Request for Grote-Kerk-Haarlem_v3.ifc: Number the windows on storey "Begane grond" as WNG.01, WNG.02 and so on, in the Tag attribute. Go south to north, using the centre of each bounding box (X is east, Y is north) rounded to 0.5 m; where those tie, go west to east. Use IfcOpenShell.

First a look at what the model holds.

```python
import ifcopenshell
import ifcopenshell.util.element
import ifcopenshell.util.placement

model = ifcopenshell.open("Grote-Kerk-Haarlem_v3.ifc")
print(model.schema)
storey = next(s for s in model.by_type("IfcBuildingStorey") if s.Name == "Begane grond")
windows = [e for e in ifcopenshell.util.element.get_decomposition(storey) if e.is_a("IfcWindow")]
for e in sorted(windows, key=lambda e: e.id()):
    origin = ifcopenshell.util.placement.get_local_placement(e.ObjectPlacement)[:3, 3]
    print(e.id(), e.Tag, e.Name, origin.round(2) + 0.0, sep=" | ")
```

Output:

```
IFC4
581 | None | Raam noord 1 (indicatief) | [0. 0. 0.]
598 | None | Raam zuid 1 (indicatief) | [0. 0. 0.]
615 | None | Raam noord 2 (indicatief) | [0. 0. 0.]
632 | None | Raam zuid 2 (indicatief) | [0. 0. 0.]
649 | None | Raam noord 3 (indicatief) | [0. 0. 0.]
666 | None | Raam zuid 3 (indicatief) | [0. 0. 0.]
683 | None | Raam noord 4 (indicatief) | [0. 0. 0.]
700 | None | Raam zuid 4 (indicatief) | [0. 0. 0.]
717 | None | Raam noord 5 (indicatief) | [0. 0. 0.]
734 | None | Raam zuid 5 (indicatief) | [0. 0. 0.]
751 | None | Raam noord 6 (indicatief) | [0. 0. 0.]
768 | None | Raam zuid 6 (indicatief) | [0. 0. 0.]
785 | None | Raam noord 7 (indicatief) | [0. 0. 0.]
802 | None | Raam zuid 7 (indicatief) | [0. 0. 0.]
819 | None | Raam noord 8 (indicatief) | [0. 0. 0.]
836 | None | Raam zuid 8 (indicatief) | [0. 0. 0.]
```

```python
import ifcopenshell
import ifcopenshell.geom
import ifcopenshell.util.element
import ifcopenshell.util.shape

model = ifcopenshell.open("Grote-Kerk-Haarlem_v3.ifc")
settings = ifcopenshell.geom.settings()
settings.set("use-world-coords", True)


def centre(element):
    shape = ifcopenshell.geom.create_shape(settings, element)
    return ifcopenshell.util.shape.get_bbox_centroid(shape.geometry)


storey = next(s for s in model.by_type("IfcBuildingStorey") if s.Name == "Begane grond")
windows = [e for e in ifcopenshell.util.element.get_decomposition(storey) if e.is_a("IfcWindow")]

# Insertion points can sit at a corner or the storey origin, so sort by the geometry (in metres).
centres = {e: centre(e) for e in windows}
windows.sort(key=lambda e: (round(centres[e][1] / 0.5), centres[e][0]))

for i, e in enumerate(windows, start=1):
    number = f"WNG.{i:02d}"
    e.Tag = number
    print(e.id(), number)

model.write("Grote-Kerk-Haarlem_v3_rev.ifc")
```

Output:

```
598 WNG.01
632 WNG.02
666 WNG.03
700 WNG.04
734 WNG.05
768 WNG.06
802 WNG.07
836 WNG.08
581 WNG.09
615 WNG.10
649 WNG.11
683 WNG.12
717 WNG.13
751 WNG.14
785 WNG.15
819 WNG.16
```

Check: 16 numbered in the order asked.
